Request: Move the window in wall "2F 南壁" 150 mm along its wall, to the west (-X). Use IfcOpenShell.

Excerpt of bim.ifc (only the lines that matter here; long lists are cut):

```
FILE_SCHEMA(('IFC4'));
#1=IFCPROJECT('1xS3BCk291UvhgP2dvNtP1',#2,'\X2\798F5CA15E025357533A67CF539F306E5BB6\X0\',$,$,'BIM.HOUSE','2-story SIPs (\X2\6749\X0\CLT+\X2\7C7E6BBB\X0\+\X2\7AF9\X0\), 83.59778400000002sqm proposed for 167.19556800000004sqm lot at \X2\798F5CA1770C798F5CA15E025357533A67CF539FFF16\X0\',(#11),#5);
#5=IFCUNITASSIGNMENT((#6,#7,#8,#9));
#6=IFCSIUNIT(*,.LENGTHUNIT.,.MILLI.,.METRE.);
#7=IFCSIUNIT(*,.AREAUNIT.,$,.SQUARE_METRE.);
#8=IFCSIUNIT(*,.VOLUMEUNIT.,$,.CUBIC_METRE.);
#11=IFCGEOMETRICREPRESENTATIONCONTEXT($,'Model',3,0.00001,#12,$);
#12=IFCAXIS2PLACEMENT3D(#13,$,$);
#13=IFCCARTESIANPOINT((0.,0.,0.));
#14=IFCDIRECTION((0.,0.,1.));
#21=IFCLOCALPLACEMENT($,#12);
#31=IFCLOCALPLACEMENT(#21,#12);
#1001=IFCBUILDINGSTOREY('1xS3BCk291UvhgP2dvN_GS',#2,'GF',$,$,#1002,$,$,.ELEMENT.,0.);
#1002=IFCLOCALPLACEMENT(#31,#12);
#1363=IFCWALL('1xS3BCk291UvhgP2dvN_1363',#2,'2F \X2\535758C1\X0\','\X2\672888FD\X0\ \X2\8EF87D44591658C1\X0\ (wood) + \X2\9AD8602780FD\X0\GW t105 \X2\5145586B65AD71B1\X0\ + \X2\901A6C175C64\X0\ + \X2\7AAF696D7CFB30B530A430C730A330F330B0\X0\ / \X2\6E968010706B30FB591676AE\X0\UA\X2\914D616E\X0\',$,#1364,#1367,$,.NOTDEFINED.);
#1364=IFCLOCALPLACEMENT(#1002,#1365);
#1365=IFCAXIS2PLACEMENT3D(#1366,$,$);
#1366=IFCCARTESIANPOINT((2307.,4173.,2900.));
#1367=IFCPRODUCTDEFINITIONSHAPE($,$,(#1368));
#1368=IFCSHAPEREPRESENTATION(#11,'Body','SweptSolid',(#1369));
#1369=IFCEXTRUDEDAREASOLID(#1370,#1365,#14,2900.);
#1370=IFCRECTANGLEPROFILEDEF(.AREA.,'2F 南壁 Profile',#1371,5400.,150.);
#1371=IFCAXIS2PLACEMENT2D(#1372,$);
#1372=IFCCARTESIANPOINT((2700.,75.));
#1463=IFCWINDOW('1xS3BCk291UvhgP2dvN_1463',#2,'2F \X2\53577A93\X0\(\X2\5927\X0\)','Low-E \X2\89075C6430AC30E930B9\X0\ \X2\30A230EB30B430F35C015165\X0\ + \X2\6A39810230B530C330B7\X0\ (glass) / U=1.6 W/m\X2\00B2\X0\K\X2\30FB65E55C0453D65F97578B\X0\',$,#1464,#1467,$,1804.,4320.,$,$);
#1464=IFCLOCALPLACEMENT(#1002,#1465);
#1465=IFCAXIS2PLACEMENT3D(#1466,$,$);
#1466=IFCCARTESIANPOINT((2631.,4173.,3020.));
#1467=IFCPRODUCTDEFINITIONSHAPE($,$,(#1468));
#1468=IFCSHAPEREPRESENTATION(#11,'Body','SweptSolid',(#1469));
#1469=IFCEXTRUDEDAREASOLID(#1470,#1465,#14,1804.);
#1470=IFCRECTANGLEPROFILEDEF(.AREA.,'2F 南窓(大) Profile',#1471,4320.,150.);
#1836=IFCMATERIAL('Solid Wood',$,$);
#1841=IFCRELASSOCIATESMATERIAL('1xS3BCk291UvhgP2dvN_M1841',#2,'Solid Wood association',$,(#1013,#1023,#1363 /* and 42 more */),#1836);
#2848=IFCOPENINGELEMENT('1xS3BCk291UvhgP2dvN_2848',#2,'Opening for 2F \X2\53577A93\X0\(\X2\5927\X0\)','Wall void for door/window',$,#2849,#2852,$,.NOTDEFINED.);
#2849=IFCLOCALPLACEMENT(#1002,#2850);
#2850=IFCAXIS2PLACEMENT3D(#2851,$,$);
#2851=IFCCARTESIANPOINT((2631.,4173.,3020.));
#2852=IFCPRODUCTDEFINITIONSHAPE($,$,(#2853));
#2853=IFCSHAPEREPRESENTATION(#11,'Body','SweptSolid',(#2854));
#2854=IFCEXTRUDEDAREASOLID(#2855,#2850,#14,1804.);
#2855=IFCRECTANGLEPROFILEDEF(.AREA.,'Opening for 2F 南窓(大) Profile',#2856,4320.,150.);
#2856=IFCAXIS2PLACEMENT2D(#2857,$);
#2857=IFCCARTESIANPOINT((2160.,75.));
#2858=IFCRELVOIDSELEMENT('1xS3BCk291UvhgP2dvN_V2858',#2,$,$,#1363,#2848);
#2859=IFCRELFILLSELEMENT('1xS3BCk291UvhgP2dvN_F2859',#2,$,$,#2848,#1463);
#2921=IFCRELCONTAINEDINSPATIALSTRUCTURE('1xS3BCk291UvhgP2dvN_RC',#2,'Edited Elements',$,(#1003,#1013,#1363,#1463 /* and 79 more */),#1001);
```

```python
import ifcopenshell
import ifcopenshell.api.geometry
import ifcopenshell.util.placement

model = ifcopenshell.open("bim.ifc")

window = model.by_guid("1xS3BCk291UvhgP2dvN_1463")
opening = window.FillsVoids[0].RelatingOpeningElement
wall = opening.VoidsElements[0].RelatingBuildingElement

wall_matrix = ifcopenshell.util.placement.get_local_placement(wall.ObjectPlacement)
shift = wall_matrix[:3, 0] * -150.0
before = ifcopenshell.util.placement.get_local_placement(window.ObjectPlacement)[:3, 3].copy()

# The window is not placed relative to its opening, so move both.
for product in (opening, window):
    matrix = ifcopenshell.util.placement.get_local_placement(product.ObjectPlacement)
    matrix[:3, 3] += shift
    ifcopenshell.api.geometry.edit_object_placement(model, product=product, matrix=matrix, is_si=False)

after = ifcopenshell.util.placement.get_local_placement(window.ObjectPlacement)[:3, 3]
print("window moved by", (after - before).round(3) + 0.0)

model.write("bim-out.ifc")
```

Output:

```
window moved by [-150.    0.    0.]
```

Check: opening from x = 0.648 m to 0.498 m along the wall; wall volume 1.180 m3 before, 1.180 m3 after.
